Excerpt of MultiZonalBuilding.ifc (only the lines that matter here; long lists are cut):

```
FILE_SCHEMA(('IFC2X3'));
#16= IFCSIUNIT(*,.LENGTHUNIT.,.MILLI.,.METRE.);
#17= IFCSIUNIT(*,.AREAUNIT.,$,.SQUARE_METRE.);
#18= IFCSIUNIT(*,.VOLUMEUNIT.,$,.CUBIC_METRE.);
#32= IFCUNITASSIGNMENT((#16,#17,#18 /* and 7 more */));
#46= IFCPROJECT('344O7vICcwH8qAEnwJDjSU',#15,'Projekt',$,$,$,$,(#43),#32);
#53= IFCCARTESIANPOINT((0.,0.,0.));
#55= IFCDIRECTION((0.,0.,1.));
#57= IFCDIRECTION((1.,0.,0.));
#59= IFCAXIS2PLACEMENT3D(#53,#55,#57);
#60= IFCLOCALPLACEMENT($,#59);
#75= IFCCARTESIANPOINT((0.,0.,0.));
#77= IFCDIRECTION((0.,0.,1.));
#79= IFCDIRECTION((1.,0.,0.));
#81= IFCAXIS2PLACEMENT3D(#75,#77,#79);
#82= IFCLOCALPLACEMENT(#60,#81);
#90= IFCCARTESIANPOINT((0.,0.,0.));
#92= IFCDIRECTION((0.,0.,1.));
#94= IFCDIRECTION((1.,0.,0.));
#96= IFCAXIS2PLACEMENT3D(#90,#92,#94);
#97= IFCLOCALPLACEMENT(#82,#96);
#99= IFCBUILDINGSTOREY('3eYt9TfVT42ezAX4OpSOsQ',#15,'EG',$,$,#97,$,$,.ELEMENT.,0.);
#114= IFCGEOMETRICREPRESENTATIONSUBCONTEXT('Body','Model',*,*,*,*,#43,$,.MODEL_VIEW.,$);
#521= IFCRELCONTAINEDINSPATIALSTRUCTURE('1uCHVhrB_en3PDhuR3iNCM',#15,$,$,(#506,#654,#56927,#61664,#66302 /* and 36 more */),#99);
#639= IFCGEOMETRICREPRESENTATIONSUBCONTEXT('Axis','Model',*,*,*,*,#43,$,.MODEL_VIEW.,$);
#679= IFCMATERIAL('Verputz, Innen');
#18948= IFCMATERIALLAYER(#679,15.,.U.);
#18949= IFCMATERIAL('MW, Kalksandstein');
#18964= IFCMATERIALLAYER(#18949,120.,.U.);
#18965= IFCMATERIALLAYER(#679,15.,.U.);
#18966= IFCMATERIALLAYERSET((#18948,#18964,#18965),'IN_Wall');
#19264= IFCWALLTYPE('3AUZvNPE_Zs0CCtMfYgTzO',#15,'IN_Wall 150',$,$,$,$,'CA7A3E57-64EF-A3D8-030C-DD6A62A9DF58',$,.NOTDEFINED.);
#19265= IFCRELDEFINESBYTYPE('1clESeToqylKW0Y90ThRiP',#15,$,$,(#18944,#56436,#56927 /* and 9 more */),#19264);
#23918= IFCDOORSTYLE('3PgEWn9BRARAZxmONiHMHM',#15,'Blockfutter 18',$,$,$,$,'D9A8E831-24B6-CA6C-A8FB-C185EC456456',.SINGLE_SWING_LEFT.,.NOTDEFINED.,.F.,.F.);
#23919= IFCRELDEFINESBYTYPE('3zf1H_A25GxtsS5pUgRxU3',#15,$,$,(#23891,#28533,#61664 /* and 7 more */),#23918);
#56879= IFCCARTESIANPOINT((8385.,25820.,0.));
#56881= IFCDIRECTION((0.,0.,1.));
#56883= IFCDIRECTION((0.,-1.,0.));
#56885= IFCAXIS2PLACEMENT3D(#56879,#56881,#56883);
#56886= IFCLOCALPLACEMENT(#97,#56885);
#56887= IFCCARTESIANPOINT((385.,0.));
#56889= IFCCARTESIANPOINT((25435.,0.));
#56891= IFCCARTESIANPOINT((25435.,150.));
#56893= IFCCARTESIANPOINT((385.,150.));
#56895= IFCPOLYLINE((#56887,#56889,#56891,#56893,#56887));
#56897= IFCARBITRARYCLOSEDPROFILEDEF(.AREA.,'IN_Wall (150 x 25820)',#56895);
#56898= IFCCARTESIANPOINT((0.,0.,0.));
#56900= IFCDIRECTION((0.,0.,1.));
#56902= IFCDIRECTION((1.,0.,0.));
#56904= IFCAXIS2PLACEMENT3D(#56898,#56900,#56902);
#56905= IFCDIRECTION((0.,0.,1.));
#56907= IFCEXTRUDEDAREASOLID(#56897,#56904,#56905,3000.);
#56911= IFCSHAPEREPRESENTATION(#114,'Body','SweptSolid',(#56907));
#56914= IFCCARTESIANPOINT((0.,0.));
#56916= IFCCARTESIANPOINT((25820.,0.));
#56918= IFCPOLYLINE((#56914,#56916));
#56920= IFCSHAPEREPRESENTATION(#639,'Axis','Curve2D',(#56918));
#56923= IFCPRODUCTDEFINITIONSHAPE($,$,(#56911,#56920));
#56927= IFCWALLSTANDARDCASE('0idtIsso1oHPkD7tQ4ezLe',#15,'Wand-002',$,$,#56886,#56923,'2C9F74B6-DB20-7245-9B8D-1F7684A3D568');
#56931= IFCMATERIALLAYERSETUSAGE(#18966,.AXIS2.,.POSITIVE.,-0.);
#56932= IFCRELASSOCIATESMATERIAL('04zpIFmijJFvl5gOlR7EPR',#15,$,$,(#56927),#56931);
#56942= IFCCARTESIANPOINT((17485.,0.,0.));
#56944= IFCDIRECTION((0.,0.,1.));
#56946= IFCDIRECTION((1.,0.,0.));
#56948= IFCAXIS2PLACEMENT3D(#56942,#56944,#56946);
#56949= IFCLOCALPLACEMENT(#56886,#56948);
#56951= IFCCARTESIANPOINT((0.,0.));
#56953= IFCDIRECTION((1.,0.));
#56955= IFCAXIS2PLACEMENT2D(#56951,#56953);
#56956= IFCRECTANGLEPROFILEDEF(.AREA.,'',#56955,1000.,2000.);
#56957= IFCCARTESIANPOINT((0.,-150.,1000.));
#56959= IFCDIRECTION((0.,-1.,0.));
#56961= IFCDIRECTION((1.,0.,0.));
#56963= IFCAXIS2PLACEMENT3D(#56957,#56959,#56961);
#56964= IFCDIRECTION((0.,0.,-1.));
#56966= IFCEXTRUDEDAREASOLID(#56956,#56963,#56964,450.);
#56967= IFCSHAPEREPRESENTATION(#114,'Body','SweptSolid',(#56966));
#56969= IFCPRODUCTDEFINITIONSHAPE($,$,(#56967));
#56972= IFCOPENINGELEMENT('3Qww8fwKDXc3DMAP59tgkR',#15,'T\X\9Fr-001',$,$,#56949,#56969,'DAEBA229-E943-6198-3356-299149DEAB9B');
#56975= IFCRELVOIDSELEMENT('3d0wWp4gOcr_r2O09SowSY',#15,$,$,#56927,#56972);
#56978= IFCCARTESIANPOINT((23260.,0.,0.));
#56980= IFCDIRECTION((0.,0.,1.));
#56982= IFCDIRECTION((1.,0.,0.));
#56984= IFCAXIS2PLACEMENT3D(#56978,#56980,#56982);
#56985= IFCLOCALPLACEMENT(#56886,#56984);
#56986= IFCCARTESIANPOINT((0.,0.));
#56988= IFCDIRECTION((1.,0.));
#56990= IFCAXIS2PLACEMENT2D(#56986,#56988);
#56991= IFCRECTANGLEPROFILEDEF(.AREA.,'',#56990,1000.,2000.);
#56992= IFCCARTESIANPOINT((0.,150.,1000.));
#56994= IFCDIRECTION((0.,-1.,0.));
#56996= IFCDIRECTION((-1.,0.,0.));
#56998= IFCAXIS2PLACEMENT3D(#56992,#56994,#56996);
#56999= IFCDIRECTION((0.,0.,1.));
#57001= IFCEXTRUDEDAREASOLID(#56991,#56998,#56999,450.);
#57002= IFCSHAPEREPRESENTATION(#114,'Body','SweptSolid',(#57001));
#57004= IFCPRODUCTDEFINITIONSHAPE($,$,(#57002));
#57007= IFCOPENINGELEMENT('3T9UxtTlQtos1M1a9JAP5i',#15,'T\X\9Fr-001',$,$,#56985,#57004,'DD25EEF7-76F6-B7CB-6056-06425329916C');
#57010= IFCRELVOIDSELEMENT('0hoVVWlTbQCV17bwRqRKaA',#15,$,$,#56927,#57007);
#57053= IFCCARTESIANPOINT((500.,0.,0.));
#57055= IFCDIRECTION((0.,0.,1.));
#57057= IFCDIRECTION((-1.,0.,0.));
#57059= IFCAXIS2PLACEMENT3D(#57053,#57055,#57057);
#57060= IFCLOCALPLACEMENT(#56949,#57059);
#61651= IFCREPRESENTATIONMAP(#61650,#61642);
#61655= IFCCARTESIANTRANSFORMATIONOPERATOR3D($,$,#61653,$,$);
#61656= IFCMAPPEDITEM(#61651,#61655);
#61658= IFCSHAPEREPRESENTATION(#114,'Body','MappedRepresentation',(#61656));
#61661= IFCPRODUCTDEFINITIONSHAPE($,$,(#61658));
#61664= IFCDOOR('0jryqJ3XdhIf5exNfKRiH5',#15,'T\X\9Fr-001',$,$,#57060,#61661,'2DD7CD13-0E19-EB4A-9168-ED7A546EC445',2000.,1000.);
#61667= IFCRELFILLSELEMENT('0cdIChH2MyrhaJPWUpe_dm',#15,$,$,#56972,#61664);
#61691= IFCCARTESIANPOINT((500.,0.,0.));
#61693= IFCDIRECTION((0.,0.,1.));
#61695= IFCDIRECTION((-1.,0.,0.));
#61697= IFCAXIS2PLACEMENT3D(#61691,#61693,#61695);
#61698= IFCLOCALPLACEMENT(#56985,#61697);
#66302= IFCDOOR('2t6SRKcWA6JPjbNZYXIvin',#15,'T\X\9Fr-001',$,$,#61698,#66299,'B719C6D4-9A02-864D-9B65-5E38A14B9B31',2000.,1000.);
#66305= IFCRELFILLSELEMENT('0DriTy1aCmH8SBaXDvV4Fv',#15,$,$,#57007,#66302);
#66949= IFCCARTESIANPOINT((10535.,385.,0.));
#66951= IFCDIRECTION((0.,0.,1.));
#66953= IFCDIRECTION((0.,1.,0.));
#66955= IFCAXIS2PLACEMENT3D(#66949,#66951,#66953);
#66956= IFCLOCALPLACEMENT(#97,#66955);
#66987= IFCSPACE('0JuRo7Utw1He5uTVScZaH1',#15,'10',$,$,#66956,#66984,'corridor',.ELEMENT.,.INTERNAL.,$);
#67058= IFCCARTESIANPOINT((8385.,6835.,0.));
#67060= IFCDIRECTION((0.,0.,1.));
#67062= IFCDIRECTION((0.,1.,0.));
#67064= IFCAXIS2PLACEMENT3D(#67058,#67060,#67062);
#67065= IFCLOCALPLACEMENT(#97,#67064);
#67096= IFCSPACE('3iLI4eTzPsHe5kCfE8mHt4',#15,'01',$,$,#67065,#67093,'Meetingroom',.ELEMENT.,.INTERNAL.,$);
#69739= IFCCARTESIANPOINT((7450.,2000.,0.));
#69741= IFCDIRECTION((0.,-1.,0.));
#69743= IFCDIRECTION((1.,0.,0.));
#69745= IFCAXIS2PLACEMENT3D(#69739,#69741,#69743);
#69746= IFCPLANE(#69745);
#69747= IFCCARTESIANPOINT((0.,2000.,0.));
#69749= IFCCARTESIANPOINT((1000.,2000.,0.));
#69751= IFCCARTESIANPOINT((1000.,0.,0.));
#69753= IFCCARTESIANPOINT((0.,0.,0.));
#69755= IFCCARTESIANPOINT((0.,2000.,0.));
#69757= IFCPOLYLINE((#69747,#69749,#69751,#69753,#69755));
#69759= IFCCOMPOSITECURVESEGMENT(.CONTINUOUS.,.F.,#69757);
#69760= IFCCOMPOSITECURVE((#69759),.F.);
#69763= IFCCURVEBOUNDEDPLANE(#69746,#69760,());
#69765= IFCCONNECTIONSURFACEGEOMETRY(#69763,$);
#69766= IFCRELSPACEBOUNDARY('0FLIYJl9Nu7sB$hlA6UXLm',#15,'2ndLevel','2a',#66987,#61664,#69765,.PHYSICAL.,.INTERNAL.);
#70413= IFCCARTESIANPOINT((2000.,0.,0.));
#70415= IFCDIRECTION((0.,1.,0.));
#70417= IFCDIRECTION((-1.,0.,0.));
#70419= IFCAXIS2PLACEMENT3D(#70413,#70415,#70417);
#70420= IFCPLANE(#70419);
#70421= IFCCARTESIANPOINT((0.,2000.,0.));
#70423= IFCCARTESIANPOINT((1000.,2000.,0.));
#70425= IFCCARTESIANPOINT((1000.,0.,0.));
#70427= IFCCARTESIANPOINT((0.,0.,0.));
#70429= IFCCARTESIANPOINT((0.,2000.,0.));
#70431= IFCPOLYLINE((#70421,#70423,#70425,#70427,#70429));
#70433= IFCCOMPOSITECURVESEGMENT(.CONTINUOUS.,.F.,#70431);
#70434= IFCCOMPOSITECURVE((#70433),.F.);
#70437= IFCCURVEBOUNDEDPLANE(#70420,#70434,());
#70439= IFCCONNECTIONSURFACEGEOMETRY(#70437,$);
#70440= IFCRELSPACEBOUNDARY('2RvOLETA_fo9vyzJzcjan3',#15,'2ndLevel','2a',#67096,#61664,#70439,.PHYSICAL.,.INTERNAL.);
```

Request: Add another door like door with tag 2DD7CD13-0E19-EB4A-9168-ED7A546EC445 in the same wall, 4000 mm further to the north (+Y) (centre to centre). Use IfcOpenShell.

```python
import numpy as np
import ifcopenshell
import ifcopenshell.api.feature
import ifcopenshell.api.geometry
import ifcopenshell.api.root
import ifcopenshell.geom
import ifcopenshell.util.element
import ifcopenshell.util.placement
import ifcopenshell.util.shape
import ifcopenshell.util.unit

model = ifcopenshell.open("MultiZonalBuilding.ifc")
unit_scale = ifcopenshell.util.unit.calculate_unit_scale(model)
settings = ifcopenshell.geom.settings()


def volume(element):
    """Net volume in cubic metres, openings subtracted."""
    shape = ifcopenshell.geom.create_shape(settings, element)
    return ifcopenshell.util.shape.get_volume(shape.geometry)


def reuse_history(source, copy):
    """copy_class also copies each property set's owner history, people and application; keep the originals."""
    for rel in copy.IsDefinedBy:
        if rel.is_a("IfcRelDefinesByProperties") and (history := rel.RelatingPropertyDefinition.OwnerHistory):
            rel.RelatingPropertyDefinition.OwnerHistory = source.OwnerHistory
            ifcopenshell.util.element.remove_deep2(model, history)


door = model.by_id(61664)
opening = door.FillsVoids[0].RelatingOpeningElement
wall = opening.VoidsElements[0].RelatingBuildingElement
before = volume(wall)
shift = ifcopenshell.util.placement.get_local_placement(wall.ObjectPlacement)[:3, 0] * -4 / unit_scale

# copy_class copies the void relationship, type, container and properties, but no geometry.
new_opening = ifcopenshell.api.root.copy_class(model, product=opening)
new_opening.Representation = ifcopenshell.util.element.copy_deep(
    model, opening.Representation, exclude=["IfcGeometricRepresentationContext", "IfcRepresentationMap"]
)
new_opening.Tag = None
new_door = ifcopenshell.api.root.copy_class(model, product=door)
new_door.Representation = ifcopenshell.util.element.copy_deep(
    model, door.Representation, exclude=["IfcGeometricRepresentationContext", "IfcRepresentationMap"]
)
new_door.Tag = None
reuse_history(door, new_door)
fills = ifcopenshell.api.feature.add_filling(model, opening=new_opening, element=new_door)
fills.OwnerHistory = new_door.OwnerHistory  # required in IFC2X3

for old, new in ((opening, new_opening), (door, new_door)):
    matrix = ifcopenshell.util.placement.get_local_placement(old.ObjectPlacement)
    matrix[:3, 3] += shift
    ifcopenshell.api.geometry.edit_object_placement(model, product=new, matrix=matrix, is_si=False)

# The copied space boundaries still share their surfaces with the original.
for rel in new_door.ProvidesBoundaries:
    if rel.ConnectionGeometry:
        rel.ConnectionGeometry = ifcopenshell.util.element.copy_deep(model, rel.ConnectionGeometry)

# Space boundary surfaces are stored in each space's coordinates; move them too.
for rel in new_door.ProvidesBoundaries:
    if not rel.ConnectionGeometry:
        continue
    surface = rel.ConnectionGeometry.SurfaceOnRelatingElement.BasisSurface
    space_matrix = ifcopenshell.util.placement.get_local_placement(rel.RelatingSpace.ObjectPlacement)
    point = np.array(surface.Position.Location.Coordinates) + space_matrix[:3, :3].T @ shift
    surface.Position = model.createIfcAxis2Placement3D(
        model.createIfcCartesianPoint(point.tolist()), surface.Position.Axis, surface.Position.RefDirection
    )

after = volume(wall)

print(f"wall volume {before:.3f} -> {after:.3f} m3")

model.write("MultiZonalBuilding_v2.ifc")
```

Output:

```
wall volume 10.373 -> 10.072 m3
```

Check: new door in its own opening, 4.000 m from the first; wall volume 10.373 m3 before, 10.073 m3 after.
